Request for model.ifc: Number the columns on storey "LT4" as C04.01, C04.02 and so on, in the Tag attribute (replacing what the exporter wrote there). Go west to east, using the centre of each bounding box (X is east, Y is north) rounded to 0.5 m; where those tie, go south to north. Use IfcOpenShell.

First a look at what the model holds.

```python
import ifcopenshell
import ifcopenshell.util.element
import ifcopenshell.util.placement

model = ifcopenshell.open("model.ifc")
print(model.schema)
storey = next(s for s in model.by_type("IfcBuildingStorey") if s.Name == "LT4")
columns = [e for e in ifcopenshell.util.element.get_decomposition(storey) if e.is_a("IfcColumn")]
for e in sorted(columns, key=lambda e: e.id()):
    origin = ifcopenshell.util.placement.get_local_placement(e.ObjectPlacement)[:3, 3]
    print(e.id(), e.Tag, e.Name, origin.round(2) + 0.0, sep=" | ")
```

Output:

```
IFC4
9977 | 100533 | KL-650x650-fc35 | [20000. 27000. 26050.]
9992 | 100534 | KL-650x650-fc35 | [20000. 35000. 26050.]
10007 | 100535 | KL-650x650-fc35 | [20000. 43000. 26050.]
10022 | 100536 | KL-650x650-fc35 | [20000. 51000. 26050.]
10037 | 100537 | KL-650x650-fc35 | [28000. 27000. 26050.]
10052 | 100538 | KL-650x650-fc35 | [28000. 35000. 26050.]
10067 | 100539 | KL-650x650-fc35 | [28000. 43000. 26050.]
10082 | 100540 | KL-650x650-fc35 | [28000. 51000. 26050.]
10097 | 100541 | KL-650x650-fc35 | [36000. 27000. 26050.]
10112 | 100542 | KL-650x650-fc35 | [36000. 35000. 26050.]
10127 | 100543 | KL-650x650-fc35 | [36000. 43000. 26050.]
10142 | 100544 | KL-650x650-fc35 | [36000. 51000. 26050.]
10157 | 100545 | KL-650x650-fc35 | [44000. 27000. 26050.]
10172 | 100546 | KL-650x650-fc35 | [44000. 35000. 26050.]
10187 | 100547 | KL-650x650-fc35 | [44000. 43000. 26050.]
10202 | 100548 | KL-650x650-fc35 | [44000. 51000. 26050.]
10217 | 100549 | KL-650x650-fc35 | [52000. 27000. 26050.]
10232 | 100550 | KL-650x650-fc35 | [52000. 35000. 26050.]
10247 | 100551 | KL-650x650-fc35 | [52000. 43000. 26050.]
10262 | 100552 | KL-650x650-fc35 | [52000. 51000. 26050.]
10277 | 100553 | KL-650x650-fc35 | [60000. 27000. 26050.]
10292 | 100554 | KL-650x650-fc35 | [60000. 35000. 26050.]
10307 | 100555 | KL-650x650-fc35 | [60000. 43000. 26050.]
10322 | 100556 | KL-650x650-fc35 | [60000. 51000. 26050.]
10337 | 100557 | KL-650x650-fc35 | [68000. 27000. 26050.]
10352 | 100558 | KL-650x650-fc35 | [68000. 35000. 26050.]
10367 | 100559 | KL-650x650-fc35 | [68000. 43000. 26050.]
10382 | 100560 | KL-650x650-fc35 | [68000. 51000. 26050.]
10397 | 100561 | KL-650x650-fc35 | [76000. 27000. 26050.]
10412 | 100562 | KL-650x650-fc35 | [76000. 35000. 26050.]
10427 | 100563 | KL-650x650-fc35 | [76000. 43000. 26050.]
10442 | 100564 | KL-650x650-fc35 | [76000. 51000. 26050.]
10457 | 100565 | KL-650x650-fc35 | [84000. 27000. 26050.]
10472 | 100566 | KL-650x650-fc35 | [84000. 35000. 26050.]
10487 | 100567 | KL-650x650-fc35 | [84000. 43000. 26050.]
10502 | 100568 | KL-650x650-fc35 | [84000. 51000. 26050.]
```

```python
import ifcopenshell
import ifcopenshell.geom
import ifcopenshell.util.element
import ifcopenshell.util.shape

model = ifcopenshell.open("model.ifc")
settings = ifcopenshell.geom.settings()
settings.set("use-world-coords", True)


def centre(element):
    shape = ifcopenshell.geom.create_shape(settings, element)
    return ifcopenshell.util.shape.get_bbox_centroid(shape.geometry)


storey = next(s for s in model.by_type("IfcBuildingStorey") if s.Name == "LT4")
columns = [e for e in ifcopenshell.util.element.get_decomposition(storey) if e.is_a("IfcColumn")]

# Insertion points can sit at a corner or the storey origin, so sort by the geometry (in metres).
centres = {e: centre(e) for e in columns}
columns.sort(key=lambda e: (round(centres[e][0] / 0.5), centres[e][1]))

for i, e in enumerate(columns, start=1):
    number = f"C04.{i:02d}"
    e.Tag = number
    print(e.id(), number)

model.write("model-out.ifc")
```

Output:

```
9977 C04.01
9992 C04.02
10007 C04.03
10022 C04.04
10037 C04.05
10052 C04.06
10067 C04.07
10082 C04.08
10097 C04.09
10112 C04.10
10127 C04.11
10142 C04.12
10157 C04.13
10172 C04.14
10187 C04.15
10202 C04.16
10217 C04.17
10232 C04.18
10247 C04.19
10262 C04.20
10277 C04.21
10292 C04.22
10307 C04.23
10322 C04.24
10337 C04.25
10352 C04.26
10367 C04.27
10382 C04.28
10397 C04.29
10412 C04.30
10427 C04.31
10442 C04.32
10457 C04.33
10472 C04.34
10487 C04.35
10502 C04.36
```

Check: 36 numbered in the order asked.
